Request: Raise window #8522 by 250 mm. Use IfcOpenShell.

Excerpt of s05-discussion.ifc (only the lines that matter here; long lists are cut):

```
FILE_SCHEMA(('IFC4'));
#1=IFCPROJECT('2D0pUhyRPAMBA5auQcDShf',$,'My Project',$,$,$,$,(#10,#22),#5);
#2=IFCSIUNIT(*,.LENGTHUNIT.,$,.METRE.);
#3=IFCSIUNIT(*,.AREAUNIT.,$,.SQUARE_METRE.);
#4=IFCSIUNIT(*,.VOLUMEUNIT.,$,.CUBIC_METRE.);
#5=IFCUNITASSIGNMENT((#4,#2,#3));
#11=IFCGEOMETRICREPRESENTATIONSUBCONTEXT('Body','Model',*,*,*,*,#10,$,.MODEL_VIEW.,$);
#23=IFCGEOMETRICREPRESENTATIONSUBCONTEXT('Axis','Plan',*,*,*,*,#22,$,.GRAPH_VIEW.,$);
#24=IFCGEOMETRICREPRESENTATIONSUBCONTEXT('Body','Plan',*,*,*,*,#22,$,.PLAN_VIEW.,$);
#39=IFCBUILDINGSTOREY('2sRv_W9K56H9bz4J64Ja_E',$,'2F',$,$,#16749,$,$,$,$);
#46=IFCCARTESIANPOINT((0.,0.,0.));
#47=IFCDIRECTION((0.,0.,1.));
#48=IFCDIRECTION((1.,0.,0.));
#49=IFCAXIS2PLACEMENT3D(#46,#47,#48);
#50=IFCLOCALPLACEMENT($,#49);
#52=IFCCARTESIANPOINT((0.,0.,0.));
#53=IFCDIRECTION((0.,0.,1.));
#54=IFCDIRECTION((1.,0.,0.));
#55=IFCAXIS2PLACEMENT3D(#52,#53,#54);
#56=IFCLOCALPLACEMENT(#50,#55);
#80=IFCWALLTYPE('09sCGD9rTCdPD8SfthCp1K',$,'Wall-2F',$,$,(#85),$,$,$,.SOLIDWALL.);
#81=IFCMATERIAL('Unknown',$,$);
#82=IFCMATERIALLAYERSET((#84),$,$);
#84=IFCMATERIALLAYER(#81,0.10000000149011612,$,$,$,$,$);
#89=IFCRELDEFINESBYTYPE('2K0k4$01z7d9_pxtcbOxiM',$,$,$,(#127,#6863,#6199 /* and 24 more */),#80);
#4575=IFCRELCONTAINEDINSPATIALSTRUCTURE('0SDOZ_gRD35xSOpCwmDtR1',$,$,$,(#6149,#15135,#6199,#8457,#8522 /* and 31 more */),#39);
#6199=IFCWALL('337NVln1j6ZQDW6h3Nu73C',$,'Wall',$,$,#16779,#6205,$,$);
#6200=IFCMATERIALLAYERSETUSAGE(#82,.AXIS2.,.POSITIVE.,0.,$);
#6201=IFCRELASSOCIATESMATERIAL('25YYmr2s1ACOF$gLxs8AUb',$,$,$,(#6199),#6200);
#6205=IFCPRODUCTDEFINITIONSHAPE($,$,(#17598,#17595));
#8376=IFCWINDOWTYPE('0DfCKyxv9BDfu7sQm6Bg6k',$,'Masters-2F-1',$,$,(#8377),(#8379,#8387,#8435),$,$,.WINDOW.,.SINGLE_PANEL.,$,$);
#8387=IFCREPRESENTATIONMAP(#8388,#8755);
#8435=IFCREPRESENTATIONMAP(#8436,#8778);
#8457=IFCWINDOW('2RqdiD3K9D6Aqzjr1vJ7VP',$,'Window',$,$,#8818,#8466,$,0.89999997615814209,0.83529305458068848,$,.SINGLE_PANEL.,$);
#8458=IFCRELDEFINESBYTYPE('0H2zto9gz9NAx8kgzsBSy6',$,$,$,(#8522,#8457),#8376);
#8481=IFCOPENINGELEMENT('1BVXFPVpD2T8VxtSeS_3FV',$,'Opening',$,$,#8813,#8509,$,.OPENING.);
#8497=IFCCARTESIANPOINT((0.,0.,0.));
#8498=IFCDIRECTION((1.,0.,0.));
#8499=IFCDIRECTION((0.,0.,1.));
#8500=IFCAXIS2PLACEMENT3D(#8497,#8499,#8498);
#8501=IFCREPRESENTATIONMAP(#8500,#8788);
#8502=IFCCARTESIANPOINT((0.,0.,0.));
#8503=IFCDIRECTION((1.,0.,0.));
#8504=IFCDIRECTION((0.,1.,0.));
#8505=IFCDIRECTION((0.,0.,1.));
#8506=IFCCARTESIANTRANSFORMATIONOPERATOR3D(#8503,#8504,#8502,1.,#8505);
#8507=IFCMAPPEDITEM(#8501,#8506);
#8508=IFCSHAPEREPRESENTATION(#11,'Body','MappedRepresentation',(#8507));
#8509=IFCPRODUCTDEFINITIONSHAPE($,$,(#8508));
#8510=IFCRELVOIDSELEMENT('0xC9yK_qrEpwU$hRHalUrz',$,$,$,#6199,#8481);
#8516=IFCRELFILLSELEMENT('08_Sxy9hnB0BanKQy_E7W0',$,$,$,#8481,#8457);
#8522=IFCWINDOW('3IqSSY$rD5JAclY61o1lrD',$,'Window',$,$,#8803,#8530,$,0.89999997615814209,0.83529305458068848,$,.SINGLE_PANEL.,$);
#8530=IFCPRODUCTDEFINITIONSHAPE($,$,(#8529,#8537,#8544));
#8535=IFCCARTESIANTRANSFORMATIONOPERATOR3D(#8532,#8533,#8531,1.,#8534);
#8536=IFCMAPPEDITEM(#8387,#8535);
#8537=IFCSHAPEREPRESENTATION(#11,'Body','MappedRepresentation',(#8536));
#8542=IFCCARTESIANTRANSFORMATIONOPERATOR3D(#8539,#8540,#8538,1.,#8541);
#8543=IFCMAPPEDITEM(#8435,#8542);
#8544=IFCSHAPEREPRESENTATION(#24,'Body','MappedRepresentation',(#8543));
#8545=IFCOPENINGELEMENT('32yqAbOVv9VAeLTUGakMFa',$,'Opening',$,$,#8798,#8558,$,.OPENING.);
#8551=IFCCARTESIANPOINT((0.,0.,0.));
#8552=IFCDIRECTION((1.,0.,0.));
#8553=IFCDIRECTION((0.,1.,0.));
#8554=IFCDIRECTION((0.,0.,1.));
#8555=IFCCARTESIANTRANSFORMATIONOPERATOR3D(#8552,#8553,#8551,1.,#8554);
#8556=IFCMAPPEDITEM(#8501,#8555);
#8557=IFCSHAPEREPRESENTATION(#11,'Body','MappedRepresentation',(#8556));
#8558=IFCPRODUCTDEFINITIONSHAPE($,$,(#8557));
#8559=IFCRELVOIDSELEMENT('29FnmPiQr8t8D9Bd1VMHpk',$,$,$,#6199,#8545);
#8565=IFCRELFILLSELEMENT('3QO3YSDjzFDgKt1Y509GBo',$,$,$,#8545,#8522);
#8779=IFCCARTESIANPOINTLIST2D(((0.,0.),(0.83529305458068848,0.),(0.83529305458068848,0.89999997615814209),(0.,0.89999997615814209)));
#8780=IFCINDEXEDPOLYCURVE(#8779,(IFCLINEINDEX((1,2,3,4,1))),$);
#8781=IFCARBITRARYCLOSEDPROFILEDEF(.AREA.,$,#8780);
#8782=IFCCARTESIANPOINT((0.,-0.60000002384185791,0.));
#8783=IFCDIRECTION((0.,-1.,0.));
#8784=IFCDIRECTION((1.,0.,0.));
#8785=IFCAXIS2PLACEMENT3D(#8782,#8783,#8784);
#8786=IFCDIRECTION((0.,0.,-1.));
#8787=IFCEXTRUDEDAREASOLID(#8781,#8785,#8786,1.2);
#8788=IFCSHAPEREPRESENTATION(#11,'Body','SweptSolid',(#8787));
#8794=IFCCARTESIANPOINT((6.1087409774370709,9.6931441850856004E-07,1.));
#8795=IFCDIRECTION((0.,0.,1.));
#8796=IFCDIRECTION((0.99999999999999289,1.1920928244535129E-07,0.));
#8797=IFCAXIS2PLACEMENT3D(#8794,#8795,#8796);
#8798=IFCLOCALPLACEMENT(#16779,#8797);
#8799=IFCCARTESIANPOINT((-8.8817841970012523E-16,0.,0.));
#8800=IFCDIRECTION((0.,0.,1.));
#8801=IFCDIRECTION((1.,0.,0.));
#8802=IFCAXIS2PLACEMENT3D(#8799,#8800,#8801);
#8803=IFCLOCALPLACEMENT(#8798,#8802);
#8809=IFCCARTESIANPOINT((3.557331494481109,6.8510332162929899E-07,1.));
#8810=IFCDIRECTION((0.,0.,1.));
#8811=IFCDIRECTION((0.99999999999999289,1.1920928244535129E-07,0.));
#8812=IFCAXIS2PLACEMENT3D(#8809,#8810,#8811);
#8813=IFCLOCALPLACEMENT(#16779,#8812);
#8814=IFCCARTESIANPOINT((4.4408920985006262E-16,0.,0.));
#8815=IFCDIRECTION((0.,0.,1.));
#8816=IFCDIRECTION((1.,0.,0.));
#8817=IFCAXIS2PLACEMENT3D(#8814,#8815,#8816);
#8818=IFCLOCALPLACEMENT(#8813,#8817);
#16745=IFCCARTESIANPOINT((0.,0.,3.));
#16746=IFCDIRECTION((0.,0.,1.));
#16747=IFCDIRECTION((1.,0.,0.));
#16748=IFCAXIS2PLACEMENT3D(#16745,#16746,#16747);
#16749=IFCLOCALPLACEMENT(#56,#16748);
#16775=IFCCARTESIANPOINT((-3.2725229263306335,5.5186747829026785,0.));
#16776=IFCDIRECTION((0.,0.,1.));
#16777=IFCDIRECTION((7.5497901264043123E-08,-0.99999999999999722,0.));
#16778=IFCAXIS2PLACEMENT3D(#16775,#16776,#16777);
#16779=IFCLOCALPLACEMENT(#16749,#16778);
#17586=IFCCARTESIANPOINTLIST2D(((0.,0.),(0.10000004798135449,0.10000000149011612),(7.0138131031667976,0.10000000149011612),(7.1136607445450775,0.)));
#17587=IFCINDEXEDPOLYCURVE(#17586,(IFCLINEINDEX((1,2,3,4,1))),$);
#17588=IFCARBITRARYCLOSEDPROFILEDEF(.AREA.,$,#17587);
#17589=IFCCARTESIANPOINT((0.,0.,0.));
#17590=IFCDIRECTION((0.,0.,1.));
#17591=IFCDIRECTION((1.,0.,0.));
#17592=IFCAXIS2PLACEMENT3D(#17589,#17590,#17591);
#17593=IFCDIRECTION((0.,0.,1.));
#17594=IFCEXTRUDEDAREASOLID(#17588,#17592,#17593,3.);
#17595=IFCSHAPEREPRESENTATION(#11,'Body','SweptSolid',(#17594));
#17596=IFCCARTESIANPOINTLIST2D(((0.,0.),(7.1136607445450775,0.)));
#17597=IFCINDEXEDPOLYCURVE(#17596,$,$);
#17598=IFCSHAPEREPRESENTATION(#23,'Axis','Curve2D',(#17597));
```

```python
import numpy as np
import ifcopenshell
import ifcopenshell.api.geometry
import ifcopenshell.util.placement
import ifcopenshell.util.unit

model = ifcopenshell.open("s05-discussion.ifc")
unit_scale = ifcopenshell.util.unit.calculate_unit_scale(model)

window = model.by_id(8522)
opening = window.FillsVoids[0].RelatingOpeningElement
dz = 0.25 / unit_scale

shift = np.array([0.0, 0.0, dz])
# The window is placed relative to its opening, so it follows when the opening moves.
matrix = ifcopenshell.util.placement.get_local_placement(opening.ObjectPlacement)
matrix[:3, 3] += shift
ifcopenshell.api.geometry.edit_object_placement(
    model, product=opening, matrix=matrix, is_si=False, should_transform_children=True
)

print(f"moved by {dz * unit_scale:+.3f} m")

model.write("s05-discussion_rev.ifc")
```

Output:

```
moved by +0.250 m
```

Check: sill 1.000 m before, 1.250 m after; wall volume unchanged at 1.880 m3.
